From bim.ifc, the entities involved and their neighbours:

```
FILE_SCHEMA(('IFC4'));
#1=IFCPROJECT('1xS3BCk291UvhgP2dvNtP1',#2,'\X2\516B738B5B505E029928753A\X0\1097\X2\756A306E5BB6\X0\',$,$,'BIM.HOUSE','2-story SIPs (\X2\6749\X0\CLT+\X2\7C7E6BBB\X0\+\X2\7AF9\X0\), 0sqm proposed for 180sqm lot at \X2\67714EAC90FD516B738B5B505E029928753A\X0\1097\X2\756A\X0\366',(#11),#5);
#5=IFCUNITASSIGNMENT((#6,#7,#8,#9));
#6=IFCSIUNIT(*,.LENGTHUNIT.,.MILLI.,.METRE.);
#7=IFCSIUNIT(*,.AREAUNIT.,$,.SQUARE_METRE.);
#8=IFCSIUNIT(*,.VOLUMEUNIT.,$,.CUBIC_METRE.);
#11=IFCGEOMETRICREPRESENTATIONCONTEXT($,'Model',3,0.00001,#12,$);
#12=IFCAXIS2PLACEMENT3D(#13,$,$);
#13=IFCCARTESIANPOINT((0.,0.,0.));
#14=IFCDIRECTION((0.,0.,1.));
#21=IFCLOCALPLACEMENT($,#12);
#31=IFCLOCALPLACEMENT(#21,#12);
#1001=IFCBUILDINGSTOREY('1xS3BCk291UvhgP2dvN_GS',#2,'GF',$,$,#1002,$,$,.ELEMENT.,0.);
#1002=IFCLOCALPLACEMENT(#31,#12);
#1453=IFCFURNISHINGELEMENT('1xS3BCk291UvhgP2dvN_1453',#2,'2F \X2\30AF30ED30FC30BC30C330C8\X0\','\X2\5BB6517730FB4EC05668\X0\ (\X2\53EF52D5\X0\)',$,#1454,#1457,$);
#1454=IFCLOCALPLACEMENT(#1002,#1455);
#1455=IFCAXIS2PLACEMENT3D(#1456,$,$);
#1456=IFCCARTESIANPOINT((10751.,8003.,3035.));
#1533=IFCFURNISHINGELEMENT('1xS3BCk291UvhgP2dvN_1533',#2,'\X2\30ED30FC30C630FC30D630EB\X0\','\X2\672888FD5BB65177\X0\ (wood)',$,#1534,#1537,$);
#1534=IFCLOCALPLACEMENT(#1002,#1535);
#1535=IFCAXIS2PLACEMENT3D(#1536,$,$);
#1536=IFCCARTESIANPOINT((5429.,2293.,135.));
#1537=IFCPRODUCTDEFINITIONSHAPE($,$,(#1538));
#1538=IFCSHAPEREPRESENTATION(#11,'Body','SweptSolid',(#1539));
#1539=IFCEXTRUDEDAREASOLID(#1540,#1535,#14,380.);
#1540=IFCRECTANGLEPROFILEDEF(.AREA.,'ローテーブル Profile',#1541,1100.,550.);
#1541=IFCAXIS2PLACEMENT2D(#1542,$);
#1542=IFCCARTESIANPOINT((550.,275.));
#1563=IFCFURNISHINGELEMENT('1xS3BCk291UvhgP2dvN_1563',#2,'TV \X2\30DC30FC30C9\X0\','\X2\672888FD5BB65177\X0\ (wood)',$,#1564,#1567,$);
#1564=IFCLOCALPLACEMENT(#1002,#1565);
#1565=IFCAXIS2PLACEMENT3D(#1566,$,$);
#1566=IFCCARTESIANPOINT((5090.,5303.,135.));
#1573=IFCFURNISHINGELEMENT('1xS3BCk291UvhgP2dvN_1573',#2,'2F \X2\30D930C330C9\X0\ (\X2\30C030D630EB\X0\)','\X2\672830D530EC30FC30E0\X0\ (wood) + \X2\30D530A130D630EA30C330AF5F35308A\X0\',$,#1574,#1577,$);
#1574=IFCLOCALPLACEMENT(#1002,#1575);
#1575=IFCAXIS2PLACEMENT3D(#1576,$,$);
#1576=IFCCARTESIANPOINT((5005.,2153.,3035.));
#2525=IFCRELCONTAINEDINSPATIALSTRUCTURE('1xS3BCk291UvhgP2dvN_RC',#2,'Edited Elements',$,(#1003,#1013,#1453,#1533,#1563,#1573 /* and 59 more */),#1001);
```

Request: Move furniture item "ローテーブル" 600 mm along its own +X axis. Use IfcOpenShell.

```python
import ifcopenshell
import ifcopenshell.api.geometry
import ifcopenshell.util.placement

model = ifcopenshell.open("bim.ifc")

item = model.by_guid("1xS3BCk291UvhgP2dvN_1533")
matrix = ifcopenshell.util.placement.get_local_placement(item.ObjectPlacement)
matrix[:3, 3] += matrix[:3, 0] * 600.0
ifcopenshell.api.geometry.edit_object_placement(model, product=item, matrix=matrix, is_si=False)

print(ifcopenshell.util.placement.get_local_placement(item.ObjectPlacement).round(3) + 0.0)

model.write("bim_edited.ifc")
```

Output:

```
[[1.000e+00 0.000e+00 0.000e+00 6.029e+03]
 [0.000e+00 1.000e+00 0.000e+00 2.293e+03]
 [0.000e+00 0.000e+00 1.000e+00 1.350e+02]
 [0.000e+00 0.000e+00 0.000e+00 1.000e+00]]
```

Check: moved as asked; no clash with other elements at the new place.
